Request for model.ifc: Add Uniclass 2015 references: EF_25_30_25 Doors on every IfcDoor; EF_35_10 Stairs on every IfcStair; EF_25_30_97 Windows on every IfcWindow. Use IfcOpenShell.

First a look at what the model holds.

```python
import ifcopenshell

model = ifcopenshell.open("model.ifc")
print(model.schema)
print("classifications:", [c.Name for c in model.by_type("IfcClassification")])
for ifc_class in ("IfcDoor", "IfcRoof", "IfcStair", "IfcWall", "IfcWindow"):
    print(ifc_class, len(model.by_type(ifc_class)))
```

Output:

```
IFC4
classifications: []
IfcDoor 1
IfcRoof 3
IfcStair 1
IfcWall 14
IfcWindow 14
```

```python
import ifcopenshell
import ifcopenshell.api.classification

model = ifcopenshell.open("model.ifc")

system = ifcopenshell.api.classification.add_classification(model, classification="Uniclass 2015")

codes = {
    "IfcDoor": ("EF_25_30_25", "Doors"),
    "IfcStair": ("EF_35_10", "Stairs"),
    "IfcWindow": ("EF_25_30_97", "Windows"),
}
for ifc_class, (code, name) in codes.items():
    products = model.by_type(ifc_class)
    ifcopenshell.api.classification.add_reference(
        model, products=products, classification=system, identification=code, name=name
    )
    print(code, len(products))

model.write("model_v2.ifc")
```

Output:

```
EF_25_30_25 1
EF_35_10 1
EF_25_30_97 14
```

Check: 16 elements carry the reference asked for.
